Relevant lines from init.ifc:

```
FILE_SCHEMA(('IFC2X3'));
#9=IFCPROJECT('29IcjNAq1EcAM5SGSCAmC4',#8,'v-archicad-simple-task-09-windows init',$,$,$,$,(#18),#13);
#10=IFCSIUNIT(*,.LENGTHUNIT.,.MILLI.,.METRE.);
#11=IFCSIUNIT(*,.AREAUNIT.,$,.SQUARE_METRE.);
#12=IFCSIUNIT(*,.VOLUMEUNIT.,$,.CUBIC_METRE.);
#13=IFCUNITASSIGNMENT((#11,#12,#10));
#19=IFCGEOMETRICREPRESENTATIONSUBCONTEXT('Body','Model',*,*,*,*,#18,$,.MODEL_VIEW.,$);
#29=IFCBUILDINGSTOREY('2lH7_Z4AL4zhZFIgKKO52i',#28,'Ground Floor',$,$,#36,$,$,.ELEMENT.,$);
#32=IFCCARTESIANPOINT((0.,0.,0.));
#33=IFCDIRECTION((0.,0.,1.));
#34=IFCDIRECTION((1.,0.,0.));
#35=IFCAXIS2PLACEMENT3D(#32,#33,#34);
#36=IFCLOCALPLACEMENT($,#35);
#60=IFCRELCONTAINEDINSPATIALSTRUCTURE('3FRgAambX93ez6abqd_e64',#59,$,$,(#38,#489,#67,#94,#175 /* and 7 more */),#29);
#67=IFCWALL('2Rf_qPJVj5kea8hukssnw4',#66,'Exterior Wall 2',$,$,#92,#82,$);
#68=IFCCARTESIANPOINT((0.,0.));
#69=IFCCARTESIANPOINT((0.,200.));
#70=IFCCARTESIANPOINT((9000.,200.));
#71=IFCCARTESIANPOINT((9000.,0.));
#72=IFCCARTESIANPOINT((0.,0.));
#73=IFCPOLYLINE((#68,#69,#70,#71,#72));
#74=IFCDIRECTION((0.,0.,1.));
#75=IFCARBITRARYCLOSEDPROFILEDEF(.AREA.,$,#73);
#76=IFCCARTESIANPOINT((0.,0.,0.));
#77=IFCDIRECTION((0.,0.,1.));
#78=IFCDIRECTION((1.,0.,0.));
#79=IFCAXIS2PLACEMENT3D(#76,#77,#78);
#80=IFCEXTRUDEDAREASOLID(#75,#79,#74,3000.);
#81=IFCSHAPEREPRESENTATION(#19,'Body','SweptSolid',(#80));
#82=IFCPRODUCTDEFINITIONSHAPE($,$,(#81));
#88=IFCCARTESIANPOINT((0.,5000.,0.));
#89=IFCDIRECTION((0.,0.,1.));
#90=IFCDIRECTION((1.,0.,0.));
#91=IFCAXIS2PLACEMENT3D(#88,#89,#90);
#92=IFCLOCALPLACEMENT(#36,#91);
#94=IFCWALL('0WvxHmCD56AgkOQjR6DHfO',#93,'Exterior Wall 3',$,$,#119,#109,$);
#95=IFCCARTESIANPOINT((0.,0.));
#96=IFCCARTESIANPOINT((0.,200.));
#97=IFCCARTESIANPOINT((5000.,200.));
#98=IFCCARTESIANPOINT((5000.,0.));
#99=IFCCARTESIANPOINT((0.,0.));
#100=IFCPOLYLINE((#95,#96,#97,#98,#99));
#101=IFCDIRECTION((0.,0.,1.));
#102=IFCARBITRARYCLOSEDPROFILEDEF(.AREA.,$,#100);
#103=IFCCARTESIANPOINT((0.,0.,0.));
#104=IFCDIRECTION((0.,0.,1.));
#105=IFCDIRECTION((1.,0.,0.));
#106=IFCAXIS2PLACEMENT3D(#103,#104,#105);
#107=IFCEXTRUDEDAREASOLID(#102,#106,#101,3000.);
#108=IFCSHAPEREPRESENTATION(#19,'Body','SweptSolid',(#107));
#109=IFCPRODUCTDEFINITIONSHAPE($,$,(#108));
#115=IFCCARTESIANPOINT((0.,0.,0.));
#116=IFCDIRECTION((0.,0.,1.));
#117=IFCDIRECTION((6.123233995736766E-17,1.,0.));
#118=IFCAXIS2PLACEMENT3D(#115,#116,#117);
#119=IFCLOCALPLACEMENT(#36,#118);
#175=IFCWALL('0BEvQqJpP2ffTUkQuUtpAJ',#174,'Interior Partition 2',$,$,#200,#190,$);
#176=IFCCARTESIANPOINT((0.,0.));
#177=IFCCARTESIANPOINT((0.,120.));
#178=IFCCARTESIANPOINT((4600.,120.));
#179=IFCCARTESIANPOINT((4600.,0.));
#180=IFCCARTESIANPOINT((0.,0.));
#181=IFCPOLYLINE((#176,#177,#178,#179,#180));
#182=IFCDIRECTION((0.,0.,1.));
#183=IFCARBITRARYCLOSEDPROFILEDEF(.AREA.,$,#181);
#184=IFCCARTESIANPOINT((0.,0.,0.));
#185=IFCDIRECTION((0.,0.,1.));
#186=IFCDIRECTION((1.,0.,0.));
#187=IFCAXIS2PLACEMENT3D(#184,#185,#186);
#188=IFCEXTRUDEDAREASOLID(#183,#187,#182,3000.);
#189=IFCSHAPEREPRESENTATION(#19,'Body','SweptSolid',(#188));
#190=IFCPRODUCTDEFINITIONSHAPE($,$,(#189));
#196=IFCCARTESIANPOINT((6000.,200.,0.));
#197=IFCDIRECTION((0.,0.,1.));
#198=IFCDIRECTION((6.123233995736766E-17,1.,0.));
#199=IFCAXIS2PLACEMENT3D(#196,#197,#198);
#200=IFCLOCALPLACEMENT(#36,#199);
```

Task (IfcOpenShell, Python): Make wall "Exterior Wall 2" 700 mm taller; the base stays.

```python
import ifcopenshell
import ifcopenshell.geom
import ifcopenshell.util.representation
import ifcopenshell.util.shape
import ifcopenshell.util.unit

model = ifcopenshell.open("init.ifc")
unit_scale = ifcopenshell.util.unit.calculate_unit_scale(model)
settings = ifcopenshell.geom.settings()


def volume(element):
    """Net volume in cubic metres, openings subtracted."""
    shape = ifcopenshell.geom.create_shape(settings, element)
    return ifcopenshell.util.shape.get_volume(shape.geometry)


wall = model.by_guid("2Rf_qPJVj5kea8hukssnw4")
before = volume(wall)

body = ifcopenshell.util.representation.get_representation(wall, "Model", "Body")
solid = body.Items[0]
old_height = solid.Depth
solid.Depth += 0.7 / unit_scale
after = volume(wall)

print(f"height {old_height:g} -> {solid.Depth:g}, volume {before:.3f} -> {after:.3f} m3")

model.write("init_updated.ifc")
```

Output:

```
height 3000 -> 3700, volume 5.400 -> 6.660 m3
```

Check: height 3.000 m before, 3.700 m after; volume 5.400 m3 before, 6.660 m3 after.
